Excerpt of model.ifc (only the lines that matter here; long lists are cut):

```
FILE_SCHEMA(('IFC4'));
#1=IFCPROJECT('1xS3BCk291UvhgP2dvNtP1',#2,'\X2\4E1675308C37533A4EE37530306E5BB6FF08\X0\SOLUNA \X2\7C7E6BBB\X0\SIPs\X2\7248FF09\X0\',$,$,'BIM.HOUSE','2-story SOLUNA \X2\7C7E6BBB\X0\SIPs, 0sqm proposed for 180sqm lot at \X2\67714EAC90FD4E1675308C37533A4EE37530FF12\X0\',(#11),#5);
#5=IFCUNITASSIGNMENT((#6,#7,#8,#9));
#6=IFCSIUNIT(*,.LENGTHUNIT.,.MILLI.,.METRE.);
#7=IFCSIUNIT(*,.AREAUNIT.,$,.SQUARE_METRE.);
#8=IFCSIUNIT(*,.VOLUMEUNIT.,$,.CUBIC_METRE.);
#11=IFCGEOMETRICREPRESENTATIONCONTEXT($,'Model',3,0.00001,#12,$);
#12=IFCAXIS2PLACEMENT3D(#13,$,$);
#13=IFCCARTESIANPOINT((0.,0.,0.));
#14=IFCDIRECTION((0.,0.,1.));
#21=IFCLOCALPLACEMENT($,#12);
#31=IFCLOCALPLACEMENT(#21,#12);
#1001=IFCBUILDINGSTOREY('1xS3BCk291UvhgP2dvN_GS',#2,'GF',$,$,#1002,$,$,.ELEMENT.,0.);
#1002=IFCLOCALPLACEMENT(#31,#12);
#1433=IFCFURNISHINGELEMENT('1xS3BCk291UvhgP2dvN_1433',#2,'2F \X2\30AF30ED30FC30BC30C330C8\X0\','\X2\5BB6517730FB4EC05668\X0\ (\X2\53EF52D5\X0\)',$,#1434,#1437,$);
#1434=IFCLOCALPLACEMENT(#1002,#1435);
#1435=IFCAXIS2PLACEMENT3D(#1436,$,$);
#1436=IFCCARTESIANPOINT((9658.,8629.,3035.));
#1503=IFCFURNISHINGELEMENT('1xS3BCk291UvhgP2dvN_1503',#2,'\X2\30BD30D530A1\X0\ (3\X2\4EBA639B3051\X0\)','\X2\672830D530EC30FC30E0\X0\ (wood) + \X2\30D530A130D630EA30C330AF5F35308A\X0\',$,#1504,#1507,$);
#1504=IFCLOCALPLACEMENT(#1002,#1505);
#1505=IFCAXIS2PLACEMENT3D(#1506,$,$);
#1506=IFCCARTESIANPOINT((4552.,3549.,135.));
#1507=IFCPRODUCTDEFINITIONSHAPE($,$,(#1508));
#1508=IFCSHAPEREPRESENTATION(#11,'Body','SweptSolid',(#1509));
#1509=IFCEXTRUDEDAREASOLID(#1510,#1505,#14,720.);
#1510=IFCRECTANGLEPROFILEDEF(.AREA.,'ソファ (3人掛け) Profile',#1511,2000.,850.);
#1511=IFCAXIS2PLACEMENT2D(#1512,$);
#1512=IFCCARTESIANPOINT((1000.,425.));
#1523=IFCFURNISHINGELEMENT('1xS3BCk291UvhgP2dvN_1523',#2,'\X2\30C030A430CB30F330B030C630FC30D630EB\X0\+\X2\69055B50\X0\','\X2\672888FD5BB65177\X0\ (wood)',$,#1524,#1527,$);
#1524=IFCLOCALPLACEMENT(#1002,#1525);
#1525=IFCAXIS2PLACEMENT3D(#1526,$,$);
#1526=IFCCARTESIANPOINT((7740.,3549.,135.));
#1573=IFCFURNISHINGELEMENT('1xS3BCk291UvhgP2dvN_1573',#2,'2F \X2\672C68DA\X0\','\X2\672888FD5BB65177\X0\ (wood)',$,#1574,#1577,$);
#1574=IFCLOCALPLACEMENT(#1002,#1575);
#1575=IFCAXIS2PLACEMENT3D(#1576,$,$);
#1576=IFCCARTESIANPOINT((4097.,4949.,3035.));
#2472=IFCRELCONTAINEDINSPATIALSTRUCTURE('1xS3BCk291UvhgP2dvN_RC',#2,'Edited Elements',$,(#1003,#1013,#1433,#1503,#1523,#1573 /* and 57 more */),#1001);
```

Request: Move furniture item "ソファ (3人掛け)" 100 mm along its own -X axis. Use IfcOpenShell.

```python
import ifcopenshell
import ifcopenshell.api.geometry
import ifcopenshell.util.placement

model = ifcopenshell.open("model.ifc")

item = model.by_guid("1xS3BCk291UvhgP2dvN_1503")
matrix = ifcopenshell.util.placement.get_local_placement(item.ObjectPlacement)
matrix[:3, 3] -= matrix[:3, 0] * 100.0
ifcopenshell.api.geometry.edit_object_placement(model, product=item, matrix=matrix, is_si=False)

print(ifcopenshell.util.placement.get_local_placement(item.ObjectPlacement).round(3) + 0.0)

model.write("model_edited.ifc")
```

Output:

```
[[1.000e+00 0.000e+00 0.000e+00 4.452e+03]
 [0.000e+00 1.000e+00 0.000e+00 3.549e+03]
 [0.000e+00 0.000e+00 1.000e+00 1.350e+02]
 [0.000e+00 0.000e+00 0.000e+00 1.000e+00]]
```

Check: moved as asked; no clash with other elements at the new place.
